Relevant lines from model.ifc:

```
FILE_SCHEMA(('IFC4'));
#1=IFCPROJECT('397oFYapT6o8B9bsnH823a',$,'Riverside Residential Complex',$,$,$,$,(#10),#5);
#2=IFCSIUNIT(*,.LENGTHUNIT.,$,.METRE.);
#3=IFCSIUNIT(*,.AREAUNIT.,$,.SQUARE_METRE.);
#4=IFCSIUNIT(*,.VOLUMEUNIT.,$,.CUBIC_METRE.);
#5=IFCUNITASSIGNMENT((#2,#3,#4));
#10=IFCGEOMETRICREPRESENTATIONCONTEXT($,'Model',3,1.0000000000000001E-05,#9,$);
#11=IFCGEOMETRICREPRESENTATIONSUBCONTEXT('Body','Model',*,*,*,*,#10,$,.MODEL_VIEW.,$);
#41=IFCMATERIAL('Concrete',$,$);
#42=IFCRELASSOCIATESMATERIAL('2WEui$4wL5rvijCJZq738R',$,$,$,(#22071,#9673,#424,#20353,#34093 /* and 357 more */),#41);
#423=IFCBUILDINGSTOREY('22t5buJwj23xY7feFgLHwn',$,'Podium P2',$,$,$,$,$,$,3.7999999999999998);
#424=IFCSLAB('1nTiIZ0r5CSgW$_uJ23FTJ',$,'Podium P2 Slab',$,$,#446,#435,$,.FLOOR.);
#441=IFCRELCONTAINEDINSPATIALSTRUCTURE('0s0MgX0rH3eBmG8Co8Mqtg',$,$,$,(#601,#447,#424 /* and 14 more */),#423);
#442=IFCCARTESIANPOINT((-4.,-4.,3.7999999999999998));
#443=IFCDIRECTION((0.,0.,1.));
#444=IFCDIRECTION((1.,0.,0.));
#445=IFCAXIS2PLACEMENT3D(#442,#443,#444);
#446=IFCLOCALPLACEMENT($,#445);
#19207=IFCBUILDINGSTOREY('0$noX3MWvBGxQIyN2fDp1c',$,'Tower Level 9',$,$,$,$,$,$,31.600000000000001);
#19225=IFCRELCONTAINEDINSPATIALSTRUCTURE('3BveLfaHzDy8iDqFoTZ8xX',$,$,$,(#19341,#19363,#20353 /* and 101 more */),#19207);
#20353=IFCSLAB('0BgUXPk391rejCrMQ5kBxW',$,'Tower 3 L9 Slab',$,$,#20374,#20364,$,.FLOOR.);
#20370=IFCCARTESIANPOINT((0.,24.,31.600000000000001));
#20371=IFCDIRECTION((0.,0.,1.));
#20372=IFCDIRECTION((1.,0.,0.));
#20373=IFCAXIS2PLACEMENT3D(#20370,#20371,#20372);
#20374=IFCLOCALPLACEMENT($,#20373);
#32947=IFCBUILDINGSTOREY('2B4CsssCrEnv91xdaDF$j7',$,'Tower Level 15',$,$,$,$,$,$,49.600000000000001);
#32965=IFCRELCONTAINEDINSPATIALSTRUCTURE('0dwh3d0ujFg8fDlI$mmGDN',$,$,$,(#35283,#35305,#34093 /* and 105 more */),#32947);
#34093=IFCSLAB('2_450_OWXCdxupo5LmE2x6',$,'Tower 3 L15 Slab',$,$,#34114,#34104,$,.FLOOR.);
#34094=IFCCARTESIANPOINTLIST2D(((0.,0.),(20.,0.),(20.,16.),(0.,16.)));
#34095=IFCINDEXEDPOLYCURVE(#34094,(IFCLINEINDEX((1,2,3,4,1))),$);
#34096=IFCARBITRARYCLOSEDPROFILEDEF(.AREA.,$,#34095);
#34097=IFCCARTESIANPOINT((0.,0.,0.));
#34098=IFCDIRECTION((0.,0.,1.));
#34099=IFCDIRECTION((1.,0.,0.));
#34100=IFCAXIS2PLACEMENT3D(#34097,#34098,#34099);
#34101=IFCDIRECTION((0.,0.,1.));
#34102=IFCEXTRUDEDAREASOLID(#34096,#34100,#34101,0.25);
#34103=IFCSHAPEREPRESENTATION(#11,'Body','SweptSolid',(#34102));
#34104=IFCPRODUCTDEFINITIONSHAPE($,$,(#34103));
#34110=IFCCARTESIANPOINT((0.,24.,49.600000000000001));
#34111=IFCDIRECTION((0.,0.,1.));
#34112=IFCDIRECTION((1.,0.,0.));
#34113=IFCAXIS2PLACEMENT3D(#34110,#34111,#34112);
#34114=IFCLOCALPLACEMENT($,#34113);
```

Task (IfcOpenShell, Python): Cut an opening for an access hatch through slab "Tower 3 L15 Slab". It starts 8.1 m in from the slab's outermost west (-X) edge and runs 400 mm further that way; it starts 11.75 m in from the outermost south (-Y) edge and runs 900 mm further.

```python
import numpy as np
import ifcopenshell
import ifcopenshell.api.feature
import ifcopenshell.api.geometry
import ifcopenshell.api.root
import ifcopenshell.geom
import ifcopenshell.util.placement
import ifcopenshell.util.representation
import ifcopenshell.util.shape
import ifcopenshell.util.unit

model = ifcopenshell.open("model.ifc")
unit_scale = ifcopenshell.util.unit.calculate_unit_scale(model)
settings = ifcopenshell.geom.settings()


def volume(element):
    """Net volume in cubic metres, openings subtracted."""
    shape = ifcopenshell.geom.create_shape(settings, element)
    return ifcopenshell.util.shape.get_volume(shape.geometry)


slab = model.by_guid("2_450_OWXCdxupo5LmE2x6")
before = volume(slab)

# Extent in the slab's own axes, in metres. The edges named are its -X and -Y sides.
slab_shape = ifcopenshell.geom.create_shape(settings, slab)
vertices = ifcopenshell.util.shape.get_vertices(slab_shape.geometry)
x_min, y_min, bottom = vertices.min(axis=0)
top = vertices[:, 2].max()

opening = ifcopenshell.api.root.create_entity(model, ifc_class="IfcOpeningElement", name="Access hatch opening", predefined_type="OPENING")
context = ifcopenshell.util.representation.get_context(model, "Model", "Body", "MODEL_VIEW")
width, depth = 0.4, 0.9
outline = [(0.0, 0.0), (width, 0.0), (width, depth), (0.0, depth), (0.0, 0.0)]
# Overshoot both faces by 50 mm so the cut is clean.
shape = ifcopenshell.api.geometry.add_slab_representation(
    model, context=context, depth=top - bottom + 0.1, polyline=outline
)
ifcopenshell.api.geometry.assign_representation(model, product=opening, representation=shape)

matrix = ifcopenshell.util.placement.get_local_placement(slab.ObjectPlacement)
matrix[:, 3] = matrix @ np.append(np.array([x_min + 8.1, y_min + 11.75, bottom - 0.05]) / unit_scale, 1.0)
ifcopenshell.api.geometry.edit_object_placement(model, product=opening, matrix=matrix, is_si=False)
ifcopenshell.api.feature.add_feature(model, feature=opening, element=slab)

after = volume(slab)

print(f"slab volume {before:.3f} -> {after:.3f} m3")

model.write("model_updated.ifc")
```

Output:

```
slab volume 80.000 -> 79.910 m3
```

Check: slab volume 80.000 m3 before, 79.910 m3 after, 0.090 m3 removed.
